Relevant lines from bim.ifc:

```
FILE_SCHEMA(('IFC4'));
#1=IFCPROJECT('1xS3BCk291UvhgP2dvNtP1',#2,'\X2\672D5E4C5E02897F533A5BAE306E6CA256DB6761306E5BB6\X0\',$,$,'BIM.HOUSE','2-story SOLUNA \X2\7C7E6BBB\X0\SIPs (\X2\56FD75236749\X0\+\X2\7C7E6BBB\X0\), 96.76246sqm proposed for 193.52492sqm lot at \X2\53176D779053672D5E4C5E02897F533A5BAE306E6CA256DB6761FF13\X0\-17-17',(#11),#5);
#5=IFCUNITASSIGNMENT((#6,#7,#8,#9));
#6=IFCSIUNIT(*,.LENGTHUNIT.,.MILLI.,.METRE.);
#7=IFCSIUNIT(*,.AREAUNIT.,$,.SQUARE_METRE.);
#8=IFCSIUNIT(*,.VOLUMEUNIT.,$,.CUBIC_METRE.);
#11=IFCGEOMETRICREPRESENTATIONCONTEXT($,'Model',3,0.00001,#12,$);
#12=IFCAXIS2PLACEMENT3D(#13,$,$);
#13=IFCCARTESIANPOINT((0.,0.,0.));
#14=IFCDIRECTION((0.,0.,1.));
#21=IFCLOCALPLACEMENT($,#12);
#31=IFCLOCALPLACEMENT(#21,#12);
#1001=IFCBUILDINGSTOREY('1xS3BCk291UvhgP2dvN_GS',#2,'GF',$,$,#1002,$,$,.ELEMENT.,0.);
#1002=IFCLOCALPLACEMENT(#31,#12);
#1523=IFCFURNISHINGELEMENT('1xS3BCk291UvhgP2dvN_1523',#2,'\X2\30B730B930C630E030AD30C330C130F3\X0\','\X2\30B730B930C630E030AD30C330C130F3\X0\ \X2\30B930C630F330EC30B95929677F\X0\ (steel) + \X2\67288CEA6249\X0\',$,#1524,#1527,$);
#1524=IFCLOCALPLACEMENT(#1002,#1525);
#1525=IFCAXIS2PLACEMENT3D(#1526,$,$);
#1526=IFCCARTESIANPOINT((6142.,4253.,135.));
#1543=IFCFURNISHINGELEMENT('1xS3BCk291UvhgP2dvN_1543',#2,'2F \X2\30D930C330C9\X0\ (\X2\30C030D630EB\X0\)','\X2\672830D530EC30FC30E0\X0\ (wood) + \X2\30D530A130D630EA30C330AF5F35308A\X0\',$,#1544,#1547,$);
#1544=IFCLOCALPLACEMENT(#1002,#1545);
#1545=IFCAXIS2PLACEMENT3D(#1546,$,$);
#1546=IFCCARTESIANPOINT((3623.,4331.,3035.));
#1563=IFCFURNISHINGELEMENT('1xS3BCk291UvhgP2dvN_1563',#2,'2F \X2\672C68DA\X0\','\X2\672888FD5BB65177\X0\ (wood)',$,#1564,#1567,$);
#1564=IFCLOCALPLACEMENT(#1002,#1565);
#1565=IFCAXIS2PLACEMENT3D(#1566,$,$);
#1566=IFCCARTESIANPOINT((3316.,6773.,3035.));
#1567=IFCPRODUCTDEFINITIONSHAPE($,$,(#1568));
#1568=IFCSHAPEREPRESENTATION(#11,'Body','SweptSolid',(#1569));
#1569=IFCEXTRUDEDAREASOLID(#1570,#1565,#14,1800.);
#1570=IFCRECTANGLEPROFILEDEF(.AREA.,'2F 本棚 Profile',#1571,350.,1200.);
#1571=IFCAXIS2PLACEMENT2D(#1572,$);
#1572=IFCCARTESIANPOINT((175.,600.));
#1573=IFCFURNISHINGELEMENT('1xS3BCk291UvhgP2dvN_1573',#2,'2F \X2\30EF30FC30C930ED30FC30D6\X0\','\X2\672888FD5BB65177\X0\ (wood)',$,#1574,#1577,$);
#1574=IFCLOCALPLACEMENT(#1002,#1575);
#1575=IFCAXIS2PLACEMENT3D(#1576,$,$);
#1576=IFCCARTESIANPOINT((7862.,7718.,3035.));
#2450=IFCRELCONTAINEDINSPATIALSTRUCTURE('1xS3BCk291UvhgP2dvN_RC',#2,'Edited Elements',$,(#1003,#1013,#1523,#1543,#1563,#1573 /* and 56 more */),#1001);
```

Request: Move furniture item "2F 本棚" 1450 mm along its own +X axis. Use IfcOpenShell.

```python
import ifcopenshell
import ifcopenshell.api.geometry
import ifcopenshell.util.placement
import ifcopenshell.util.unit

model = ifcopenshell.open("bim.ifc")
unit_scale = ifcopenshell.util.unit.calculate_unit_scale(model)

item = model.by_guid("1xS3BCk291UvhgP2dvN_1563")
matrix = ifcopenshell.util.placement.get_local_placement(item.ObjectPlacement)
matrix[:3, 3] += matrix[:3, 0] * 1.45 / unit_scale
ifcopenshell.api.geometry.edit_object_placement(model, product=item, matrix=matrix, is_si=False)

print(ifcopenshell.util.placement.get_local_placement(item.ObjectPlacement).round(3) + 0.0)

model.write("bim_edited.ifc")
```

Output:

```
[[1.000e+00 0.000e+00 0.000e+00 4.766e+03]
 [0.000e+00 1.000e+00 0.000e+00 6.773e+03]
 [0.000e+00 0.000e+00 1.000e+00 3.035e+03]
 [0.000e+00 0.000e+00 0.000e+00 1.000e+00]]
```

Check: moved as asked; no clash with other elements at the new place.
